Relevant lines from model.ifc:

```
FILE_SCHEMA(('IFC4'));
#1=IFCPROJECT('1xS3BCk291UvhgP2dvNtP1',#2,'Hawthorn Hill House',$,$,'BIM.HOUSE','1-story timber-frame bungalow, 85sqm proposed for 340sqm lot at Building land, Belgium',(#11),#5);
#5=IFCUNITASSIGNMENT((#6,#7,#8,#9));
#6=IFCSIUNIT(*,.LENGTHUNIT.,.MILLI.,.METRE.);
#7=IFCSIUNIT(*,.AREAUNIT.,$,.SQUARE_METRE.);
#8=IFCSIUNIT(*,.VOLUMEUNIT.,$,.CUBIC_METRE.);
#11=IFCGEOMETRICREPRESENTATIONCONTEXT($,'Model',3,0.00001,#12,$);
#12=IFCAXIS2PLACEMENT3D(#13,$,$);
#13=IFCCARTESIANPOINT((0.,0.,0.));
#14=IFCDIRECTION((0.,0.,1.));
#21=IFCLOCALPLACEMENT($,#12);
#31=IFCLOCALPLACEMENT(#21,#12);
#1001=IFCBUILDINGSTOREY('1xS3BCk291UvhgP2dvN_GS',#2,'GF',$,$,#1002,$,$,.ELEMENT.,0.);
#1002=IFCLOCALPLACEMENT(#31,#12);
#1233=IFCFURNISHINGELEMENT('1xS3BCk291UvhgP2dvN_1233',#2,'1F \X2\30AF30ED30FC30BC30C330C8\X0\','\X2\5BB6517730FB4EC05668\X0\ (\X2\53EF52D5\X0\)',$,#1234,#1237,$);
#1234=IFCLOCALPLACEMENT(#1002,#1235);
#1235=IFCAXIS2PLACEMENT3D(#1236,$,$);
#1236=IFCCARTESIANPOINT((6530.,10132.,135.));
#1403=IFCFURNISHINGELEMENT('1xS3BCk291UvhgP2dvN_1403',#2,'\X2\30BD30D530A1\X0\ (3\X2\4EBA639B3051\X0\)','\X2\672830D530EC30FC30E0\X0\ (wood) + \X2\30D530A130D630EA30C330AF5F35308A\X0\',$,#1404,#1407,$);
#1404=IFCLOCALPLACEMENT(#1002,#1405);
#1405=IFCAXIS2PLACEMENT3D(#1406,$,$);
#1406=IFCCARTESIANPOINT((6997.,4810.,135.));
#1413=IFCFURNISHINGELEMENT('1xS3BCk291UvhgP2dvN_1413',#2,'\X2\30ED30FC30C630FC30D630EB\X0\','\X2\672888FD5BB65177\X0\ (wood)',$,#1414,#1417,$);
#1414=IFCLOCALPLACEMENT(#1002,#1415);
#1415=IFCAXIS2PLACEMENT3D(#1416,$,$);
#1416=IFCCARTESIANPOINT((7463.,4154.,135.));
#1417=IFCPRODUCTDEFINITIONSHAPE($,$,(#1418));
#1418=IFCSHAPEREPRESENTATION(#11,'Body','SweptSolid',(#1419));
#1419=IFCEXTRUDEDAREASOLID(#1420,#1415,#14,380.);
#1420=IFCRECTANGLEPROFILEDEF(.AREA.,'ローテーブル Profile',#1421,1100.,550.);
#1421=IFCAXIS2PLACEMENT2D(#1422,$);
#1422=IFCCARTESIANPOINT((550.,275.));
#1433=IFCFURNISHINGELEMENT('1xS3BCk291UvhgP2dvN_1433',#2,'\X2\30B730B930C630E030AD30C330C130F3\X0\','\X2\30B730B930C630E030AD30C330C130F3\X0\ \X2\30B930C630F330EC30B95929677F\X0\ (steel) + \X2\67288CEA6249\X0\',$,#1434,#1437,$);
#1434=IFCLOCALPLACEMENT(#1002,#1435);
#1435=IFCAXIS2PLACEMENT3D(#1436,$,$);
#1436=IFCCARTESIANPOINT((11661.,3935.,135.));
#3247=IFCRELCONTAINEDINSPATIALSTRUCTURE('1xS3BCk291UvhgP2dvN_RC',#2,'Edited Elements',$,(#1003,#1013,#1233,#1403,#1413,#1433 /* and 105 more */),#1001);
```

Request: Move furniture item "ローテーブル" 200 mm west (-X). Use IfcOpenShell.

```python
import ifcopenshell
import ifcopenshell.api.geometry
import ifcopenshell.util.placement

model = ifcopenshell.open("model.ifc")

item = model.by_guid("1xS3BCk291UvhgP2dvN_1413")
matrix = ifcopenshell.util.placement.get_local_placement(item.ObjectPlacement)
matrix[0, 3] -= 200.0
ifcopenshell.api.geometry.edit_object_placement(model, product=item, matrix=matrix, is_si=False)

print(ifcopenshell.util.placement.get_local_placement(item.ObjectPlacement).round(3) + 0.0)

model.write("model-out.ifc")
```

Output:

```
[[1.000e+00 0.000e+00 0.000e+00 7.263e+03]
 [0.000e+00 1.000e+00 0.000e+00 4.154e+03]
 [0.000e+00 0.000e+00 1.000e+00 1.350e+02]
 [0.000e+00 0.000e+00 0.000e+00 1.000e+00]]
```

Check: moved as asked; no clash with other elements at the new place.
